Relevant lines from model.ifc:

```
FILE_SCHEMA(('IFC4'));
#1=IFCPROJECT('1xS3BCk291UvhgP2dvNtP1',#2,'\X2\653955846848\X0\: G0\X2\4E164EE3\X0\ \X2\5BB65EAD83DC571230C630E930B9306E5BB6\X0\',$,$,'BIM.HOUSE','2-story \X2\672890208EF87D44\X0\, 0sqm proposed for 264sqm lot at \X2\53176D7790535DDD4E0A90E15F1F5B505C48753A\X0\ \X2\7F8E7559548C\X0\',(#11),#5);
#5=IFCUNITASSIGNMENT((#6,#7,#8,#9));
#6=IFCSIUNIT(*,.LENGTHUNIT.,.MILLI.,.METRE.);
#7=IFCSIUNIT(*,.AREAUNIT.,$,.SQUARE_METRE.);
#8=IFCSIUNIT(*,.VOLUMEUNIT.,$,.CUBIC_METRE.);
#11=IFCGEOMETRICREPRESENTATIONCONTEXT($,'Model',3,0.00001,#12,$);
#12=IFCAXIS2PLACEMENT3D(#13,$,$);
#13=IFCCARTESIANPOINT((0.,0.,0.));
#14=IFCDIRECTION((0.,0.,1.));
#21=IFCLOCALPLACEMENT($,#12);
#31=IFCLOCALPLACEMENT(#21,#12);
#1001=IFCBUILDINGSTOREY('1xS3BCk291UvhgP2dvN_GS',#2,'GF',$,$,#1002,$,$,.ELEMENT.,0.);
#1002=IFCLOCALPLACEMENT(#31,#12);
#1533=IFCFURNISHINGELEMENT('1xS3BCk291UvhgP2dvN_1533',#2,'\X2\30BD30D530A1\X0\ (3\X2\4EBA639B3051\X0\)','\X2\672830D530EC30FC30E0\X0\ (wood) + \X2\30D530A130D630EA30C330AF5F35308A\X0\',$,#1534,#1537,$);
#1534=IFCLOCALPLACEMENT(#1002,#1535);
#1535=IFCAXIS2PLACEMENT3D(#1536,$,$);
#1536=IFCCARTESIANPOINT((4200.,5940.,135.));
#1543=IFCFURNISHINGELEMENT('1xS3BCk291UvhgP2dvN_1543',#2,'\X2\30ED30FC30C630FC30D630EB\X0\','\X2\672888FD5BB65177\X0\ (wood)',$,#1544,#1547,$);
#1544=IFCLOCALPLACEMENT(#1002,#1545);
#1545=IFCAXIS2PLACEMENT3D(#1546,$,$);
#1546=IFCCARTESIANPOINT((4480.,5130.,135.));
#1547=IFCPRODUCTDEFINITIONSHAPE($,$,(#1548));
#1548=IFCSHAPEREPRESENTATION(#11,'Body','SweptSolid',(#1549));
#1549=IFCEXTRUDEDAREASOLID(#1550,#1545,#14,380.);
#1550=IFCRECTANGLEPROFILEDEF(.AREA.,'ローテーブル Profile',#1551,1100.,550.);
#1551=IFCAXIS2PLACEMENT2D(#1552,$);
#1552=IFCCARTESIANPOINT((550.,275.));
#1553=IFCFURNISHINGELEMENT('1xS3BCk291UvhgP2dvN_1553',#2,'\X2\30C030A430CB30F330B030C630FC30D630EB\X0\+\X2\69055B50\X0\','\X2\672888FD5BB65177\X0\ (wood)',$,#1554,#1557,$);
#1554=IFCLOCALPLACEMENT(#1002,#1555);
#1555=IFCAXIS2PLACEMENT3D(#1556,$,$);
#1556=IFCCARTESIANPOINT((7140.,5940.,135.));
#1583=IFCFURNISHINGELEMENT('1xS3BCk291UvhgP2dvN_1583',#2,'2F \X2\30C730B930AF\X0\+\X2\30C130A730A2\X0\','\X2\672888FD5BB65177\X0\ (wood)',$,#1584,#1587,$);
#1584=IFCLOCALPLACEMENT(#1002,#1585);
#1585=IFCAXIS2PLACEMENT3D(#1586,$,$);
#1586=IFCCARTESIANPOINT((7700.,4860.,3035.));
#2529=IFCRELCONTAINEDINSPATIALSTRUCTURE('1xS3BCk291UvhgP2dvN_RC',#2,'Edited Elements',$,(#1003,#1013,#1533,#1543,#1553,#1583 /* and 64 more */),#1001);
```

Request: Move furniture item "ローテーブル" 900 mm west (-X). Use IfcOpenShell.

```python
import ifcopenshell
import ifcopenshell.api.geometry
import ifcopenshell.util.placement

model = ifcopenshell.open("model.ifc")

item = model.by_guid("1xS3BCk291UvhgP2dvN_1543")
matrix = ifcopenshell.util.placement.get_local_placement(item.ObjectPlacement)
matrix[0, 3] -= 900.0
ifcopenshell.api.geometry.edit_object_placement(model, product=item, matrix=matrix, is_si=False)

print(ifcopenshell.util.placement.get_local_placement(item.ObjectPlacement).round(3) + 0.0)

model.write("model_edited.ifc")
```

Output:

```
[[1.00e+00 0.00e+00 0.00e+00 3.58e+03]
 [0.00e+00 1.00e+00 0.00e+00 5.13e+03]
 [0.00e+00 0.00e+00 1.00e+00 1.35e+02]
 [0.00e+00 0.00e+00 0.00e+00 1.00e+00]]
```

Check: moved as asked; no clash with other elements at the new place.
